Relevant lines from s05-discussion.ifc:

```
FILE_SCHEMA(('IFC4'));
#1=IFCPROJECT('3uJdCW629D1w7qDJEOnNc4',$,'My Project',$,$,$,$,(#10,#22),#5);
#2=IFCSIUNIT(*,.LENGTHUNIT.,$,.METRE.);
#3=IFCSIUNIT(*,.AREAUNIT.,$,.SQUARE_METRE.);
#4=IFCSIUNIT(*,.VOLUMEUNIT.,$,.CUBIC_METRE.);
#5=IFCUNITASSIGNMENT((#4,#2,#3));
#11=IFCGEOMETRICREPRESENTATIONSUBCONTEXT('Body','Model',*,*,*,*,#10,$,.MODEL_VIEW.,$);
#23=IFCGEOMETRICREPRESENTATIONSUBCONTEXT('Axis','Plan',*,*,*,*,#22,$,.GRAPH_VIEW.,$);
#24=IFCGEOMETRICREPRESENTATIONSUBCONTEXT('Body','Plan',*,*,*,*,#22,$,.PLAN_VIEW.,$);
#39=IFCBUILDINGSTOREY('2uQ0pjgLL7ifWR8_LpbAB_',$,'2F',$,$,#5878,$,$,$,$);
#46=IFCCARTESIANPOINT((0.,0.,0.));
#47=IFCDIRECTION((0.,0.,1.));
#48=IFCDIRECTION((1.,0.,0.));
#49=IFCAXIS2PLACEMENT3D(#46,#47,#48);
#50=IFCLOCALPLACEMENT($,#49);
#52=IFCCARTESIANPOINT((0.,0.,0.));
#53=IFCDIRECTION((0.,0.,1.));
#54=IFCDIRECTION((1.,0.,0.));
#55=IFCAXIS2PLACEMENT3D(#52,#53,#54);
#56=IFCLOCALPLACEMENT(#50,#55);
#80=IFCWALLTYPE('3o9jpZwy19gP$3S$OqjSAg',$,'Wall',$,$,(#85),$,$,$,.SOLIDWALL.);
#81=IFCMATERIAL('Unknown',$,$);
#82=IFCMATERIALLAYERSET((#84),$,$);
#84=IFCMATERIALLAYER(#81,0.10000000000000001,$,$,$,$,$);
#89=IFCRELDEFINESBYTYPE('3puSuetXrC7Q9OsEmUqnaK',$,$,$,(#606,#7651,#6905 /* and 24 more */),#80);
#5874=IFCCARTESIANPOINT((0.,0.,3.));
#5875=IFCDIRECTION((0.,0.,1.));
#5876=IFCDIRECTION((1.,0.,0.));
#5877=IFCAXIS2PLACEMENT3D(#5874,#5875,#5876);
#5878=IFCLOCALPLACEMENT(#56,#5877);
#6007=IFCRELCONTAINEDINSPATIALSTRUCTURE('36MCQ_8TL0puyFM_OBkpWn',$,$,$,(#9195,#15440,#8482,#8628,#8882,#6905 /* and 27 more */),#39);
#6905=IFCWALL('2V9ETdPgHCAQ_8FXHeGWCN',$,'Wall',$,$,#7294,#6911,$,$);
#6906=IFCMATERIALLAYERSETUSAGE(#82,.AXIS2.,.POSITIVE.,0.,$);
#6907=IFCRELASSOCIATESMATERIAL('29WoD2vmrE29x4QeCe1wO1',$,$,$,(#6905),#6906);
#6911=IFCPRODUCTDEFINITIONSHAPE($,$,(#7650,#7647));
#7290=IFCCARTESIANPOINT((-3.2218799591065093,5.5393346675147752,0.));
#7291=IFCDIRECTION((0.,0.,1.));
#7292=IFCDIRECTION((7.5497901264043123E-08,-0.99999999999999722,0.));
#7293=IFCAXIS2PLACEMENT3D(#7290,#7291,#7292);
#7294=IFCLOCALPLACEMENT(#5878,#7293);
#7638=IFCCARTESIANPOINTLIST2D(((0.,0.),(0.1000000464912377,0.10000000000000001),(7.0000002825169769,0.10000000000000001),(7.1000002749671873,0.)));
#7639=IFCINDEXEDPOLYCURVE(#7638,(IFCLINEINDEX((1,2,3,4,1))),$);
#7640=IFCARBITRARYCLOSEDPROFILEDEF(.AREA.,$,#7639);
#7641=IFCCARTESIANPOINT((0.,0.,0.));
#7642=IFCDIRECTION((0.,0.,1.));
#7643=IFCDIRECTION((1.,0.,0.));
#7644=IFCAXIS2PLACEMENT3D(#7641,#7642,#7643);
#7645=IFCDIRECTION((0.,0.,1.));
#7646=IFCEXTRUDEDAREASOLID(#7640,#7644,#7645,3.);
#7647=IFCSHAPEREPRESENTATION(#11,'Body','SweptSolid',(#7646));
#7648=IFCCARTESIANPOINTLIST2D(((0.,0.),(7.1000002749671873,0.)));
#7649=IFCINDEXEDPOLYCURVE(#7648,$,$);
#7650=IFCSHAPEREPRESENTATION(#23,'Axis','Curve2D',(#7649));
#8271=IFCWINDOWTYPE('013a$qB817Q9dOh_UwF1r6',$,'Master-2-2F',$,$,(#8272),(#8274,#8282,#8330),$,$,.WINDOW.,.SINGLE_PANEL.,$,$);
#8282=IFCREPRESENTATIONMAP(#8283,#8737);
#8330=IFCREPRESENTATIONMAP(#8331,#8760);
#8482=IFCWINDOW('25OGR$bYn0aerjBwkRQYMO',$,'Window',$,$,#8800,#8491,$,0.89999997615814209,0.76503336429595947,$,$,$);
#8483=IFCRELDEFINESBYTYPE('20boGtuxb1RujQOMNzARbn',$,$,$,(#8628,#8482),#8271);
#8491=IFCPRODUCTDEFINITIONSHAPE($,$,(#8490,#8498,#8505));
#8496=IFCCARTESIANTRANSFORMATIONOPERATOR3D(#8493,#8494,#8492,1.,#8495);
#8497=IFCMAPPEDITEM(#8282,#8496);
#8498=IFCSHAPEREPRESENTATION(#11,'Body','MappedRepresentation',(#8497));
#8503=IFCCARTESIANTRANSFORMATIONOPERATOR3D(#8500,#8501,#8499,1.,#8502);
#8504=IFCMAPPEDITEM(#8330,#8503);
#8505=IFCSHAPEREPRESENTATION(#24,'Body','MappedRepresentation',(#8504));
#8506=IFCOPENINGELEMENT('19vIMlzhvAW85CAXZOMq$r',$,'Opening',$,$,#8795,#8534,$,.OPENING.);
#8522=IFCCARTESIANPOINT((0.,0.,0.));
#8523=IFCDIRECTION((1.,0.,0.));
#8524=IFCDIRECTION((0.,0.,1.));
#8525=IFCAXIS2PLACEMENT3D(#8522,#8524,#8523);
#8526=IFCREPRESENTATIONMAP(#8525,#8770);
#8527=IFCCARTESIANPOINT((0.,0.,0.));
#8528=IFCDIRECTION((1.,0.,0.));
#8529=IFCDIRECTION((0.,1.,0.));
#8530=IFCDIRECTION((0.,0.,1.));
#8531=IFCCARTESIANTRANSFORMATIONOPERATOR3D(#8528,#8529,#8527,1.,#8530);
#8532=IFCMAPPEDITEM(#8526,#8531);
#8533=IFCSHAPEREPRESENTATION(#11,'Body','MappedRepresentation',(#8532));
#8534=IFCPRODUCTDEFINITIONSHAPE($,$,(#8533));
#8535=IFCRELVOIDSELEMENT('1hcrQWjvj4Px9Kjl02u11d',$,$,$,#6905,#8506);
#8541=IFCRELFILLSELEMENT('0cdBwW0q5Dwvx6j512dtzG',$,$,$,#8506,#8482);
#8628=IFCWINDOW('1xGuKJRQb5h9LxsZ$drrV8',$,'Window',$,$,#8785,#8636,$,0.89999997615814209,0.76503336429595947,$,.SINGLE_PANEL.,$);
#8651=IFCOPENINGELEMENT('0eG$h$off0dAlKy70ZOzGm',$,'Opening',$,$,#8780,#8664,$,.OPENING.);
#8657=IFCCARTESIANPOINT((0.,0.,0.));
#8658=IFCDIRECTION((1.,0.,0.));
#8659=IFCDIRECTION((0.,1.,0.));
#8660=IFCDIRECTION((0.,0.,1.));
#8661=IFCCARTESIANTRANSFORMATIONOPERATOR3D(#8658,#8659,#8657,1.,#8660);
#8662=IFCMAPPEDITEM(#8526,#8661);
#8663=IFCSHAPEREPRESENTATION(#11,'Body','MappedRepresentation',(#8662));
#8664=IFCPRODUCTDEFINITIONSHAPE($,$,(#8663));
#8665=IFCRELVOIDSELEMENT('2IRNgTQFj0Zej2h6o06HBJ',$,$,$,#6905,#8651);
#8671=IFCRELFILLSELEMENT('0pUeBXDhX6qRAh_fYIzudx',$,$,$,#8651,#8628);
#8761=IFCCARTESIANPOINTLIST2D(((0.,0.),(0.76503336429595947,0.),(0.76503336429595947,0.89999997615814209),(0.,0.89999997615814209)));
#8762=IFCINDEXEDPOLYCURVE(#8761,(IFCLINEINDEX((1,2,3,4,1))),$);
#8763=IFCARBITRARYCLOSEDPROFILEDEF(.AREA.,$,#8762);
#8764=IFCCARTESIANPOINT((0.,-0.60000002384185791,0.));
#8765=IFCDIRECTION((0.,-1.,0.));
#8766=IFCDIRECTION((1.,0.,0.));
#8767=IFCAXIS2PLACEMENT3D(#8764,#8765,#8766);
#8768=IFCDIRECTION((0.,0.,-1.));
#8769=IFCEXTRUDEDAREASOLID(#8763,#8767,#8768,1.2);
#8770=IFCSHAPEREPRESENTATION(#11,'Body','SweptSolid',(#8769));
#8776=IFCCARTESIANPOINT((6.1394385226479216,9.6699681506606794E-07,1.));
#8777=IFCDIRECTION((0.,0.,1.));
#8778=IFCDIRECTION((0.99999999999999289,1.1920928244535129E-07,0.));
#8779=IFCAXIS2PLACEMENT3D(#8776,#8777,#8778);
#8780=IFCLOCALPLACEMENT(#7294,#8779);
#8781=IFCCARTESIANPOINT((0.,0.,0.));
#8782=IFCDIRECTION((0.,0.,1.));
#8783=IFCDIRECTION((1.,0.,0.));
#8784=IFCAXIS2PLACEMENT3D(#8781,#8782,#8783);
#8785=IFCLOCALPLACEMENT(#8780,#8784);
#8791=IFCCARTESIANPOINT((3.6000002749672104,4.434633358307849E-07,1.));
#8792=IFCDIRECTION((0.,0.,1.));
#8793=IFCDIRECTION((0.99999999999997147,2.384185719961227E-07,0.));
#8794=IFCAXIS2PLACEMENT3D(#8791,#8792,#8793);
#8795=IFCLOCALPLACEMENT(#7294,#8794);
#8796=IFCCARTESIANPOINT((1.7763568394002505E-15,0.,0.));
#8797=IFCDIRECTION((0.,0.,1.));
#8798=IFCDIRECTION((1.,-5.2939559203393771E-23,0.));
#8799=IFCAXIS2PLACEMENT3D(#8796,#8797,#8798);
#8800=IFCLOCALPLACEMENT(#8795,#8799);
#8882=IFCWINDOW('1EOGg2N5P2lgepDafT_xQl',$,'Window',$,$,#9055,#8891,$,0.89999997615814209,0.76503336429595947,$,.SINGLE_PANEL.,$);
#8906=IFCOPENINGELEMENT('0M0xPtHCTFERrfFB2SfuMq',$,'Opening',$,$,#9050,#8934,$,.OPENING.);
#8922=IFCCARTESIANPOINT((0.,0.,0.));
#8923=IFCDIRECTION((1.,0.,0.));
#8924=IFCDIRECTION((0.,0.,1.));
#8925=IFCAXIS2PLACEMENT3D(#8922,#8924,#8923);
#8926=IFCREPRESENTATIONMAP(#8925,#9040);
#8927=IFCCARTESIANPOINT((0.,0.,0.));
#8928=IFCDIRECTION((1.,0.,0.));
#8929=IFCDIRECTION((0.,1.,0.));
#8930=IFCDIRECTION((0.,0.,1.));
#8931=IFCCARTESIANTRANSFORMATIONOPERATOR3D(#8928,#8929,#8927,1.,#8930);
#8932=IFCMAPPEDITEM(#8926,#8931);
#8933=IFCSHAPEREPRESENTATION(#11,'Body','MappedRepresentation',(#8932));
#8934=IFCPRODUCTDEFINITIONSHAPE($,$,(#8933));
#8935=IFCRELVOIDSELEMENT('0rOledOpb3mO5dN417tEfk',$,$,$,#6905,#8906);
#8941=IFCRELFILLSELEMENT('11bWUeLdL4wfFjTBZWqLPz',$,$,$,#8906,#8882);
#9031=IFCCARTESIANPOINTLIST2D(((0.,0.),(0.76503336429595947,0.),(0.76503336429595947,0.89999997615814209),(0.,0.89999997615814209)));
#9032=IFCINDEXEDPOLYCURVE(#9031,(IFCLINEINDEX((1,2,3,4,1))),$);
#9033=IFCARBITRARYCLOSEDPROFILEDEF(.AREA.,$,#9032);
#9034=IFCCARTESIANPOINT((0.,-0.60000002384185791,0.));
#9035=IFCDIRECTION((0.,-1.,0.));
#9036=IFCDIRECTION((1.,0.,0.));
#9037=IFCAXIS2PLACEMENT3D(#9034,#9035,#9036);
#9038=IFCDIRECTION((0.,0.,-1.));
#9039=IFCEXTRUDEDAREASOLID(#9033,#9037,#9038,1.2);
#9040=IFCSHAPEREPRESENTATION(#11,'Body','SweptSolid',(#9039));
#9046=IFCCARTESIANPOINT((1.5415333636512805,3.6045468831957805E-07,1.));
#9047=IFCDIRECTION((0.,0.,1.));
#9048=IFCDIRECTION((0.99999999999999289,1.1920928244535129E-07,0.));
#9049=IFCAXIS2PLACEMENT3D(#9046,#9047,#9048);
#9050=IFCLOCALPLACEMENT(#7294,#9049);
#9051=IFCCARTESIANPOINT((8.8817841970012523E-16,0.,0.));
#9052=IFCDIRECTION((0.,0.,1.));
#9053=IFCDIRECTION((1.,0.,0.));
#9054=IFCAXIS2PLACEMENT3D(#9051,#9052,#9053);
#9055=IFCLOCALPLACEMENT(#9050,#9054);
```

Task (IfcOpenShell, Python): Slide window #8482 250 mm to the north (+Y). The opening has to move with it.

```python
import ifcopenshell
import ifcopenshell.api.geometry
import ifcopenshell.util.placement

model = ifcopenshell.open("s05-discussion.ifc")

window = model.by_id(8482)
opening = window.FillsVoids[0].RelatingOpeningElement
wall = opening.VoidsElements[0].RelatingBuildingElement

wall_matrix = ifcopenshell.util.placement.get_local_placement(wall.ObjectPlacement)
shift = wall_matrix[:3, 0] * -0.25
before = ifcopenshell.util.placement.get_local_placement(window.ObjectPlacement)[:3, 3].copy()

# The window is placed relative to its opening, so it follows when the opening moves.
matrix = ifcopenshell.util.placement.get_local_placement(opening.ObjectPlacement)
matrix[:3, 3] += shift
ifcopenshell.api.geometry.edit_object_placement(
    model, product=opening, matrix=matrix, is_si=False, should_transform_children=True
)

after = ifcopenshell.util.placement.get_local_placement(window.ObjectPlacement)[:3, 3]
print("window moved by", (after - before).round(3) + 0.0)

model.write("s05-discussion_v2.ifc")
```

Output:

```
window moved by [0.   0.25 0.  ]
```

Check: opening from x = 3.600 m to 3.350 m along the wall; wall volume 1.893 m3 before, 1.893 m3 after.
